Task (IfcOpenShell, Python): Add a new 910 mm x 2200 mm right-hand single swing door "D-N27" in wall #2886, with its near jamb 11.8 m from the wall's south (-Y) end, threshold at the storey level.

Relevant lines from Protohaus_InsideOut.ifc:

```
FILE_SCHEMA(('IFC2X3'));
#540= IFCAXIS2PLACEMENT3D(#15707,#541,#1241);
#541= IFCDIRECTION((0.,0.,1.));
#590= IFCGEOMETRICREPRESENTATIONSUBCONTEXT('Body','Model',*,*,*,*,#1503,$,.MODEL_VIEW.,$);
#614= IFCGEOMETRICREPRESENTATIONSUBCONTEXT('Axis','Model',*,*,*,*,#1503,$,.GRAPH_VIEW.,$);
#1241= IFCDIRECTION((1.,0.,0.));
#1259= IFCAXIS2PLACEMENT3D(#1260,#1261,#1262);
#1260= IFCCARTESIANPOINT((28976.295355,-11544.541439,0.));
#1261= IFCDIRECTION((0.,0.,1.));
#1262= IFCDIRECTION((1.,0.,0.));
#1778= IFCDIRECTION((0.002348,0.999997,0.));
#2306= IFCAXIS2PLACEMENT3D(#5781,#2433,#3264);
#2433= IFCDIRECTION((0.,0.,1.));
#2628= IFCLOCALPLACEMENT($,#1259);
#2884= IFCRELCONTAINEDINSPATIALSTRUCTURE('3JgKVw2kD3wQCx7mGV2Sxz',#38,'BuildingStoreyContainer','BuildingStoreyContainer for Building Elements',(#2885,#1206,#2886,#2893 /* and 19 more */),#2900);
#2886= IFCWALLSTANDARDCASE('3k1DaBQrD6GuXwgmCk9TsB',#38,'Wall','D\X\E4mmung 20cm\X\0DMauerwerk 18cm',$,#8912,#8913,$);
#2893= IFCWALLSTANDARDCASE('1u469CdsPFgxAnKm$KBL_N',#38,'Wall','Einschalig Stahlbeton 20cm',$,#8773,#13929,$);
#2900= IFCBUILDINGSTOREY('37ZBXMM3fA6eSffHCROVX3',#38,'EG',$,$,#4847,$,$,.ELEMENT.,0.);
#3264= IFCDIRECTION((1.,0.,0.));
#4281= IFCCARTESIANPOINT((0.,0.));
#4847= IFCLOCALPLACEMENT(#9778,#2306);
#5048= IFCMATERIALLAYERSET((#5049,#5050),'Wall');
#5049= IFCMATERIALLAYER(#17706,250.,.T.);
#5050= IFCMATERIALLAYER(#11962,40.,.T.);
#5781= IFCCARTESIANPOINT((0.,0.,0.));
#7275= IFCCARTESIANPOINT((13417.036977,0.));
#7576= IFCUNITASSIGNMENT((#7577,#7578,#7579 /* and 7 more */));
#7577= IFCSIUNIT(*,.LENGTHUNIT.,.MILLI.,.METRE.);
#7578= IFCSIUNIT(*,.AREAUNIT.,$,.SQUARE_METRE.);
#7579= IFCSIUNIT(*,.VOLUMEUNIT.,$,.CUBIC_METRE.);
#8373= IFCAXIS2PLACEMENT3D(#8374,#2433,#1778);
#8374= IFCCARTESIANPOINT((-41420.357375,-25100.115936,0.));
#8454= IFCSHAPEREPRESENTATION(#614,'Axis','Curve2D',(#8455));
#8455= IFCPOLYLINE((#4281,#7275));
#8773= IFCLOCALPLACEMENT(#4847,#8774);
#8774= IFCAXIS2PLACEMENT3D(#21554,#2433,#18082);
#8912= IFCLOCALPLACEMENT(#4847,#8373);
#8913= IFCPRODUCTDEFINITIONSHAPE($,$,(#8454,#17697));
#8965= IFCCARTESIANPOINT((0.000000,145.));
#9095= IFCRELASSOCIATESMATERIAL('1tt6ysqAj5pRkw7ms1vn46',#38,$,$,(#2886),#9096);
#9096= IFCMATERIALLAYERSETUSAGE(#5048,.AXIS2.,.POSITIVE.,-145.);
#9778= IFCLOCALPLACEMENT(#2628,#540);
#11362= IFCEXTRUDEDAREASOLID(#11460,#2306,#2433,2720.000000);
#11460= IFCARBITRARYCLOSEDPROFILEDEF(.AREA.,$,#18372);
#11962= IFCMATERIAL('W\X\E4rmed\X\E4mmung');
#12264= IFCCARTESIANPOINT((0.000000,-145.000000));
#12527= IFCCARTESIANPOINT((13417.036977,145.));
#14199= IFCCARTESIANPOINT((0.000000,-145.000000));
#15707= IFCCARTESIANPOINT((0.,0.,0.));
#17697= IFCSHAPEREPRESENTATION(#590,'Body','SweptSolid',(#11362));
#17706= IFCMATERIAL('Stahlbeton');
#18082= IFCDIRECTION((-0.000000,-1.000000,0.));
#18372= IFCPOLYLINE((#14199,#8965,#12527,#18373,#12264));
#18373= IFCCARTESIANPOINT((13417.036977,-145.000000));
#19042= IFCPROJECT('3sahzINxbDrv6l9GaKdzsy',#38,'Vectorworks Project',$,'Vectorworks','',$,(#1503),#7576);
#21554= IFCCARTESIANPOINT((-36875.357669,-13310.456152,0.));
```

```python
import numpy as np
import ifcopenshell
import ifcopenshell.api.feature
import ifcopenshell.api.geometry
import ifcopenshell.api.root
import ifcopenshell.api.spatial
import ifcopenshell.api.type
import ifcopenshell.geom
import ifcopenshell.util.element
import ifcopenshell.util.placement
import ifcopenshell.util.representation
import ifcopenshell.util.shape
import ifcopenshell.util.unit

model = ifcopenshell.open("Protohaus_InsideOut.ifc")
unit_scale = ifcopenshell.util.unit.calculate_unit_scale(model)
settings = ifcopenshell.geom.settings()


def volume(element):
    """Net volume in cubic metres, openings subtracted."""
    shape = ifcopenshell.geom.create_shape(settings, element)
    return ifcopenshell.util.shape.get_volume(shape.geometry)


wall = model.by_guid("3k1DaBQrD6GuXwgmCk9TsB")
storey = ifcopenshell.util.element.get_container(wall, ifc_class="IfcBuildingStorey")
context = ifcopenshell.util.representation.get_context(model, "Model", "Body", "MODEL_VIEW")
before = volume(wall)

width, height, from_end, sill = 0.91, 2.2, 11.8, 0.0  # metres

# The wall runs along its own X axis, and the end named is its -X end.
wall_shape = ifcopenshell.geom.create_shape(settings, wall)
x, y, z = ifcopenshell.util.shape.get_vertices(wall_shape.geometry).T
start = x.min() + from_end
face, thickness = float(y.min()), float(y.max() - y.min())
wall_matrix = ifcopenshell.util.placement.get_local_placement(wall.ObjectPlacement)
level = ifcopenshell.util.placement.get_local_placement(storey.ObjectPlacement)[2, 3]


def in_wall(x, y):
    """Placement at x, y metres in the wall's axes, at sill height."""
    matrix = wall_matrix.copy()
    matrix[:, 3] = wall_matrix @ np.array([x / unit_scale, y / unit_scale, 0.0, 1.0])
    matrix[2, 3] = level + sill / unit_scale
    return matrix


# Opening: a box that overshoots both wall faces by 50 mm.
opening = ifcopenshell.api.root.create_entity(model, ifc_class="IfcOpeningElement")
box = ifcopenshell.api.geometry.add_wall_representation(
    model, context=context, length=width, height=height, thickness=thickness + 0.1
)
ifcopenshell.api.geometry.assign_representation(model, product=opening, representation=box)
ifcopenshell.api.geometry.edit_object_placement(model, product=opening, matrix=in_wall(start, face - 0.05), is_si=False)
ifcopenshell.api.feature.add_feature(model, feature=opening, element=wall)

door = ifcopenshell.api.root.create_entity(model, ifc_class="IfcDoor", name="D-N27")
door.OverallWidth, door.OverallHeight = width / unit_scale, height / unit_scale
body = ifcopenshell.api.geometry.add_door_representation(
    model,
    context=context,
    overall_width=door.OverallWidth,
    overall_height=door.OverallHeight,
    operation_type="SINGLE_SWING_RIGHT",
    lining_properties={"LiningDepth": thickness / unit_scale, "ThresholdDepth": thickness / unit_scale},
)
ifcopenshell.api.geometry.assign_representation(model, product=door, representation=body)
ifcopenshell.api.spatial.assign_container(model, products=[door], relating_structure=storey)
fills = ifcopenshell.api.feature.add_filling(model, opening=opening, element=door)
fills.OwnerHistory = door.OwnerHistory  # required in IFC2X3

# IFC2X3 keeps the operation on the door style.
style = ifcopenshell.api.root.create_entity(model, ifc_class="IfcDoorStyle", name="D-N27")
style.OperationType, style.ConstructionType = "SINGLE_SWING_RIGHT", "NOTDEFINED"
style.ParameterTakesPrecedence = style.Sizeable = False
ifcopenshell.api.type.assign_type(model, related_objects=[door], relating_type=style)

# The lining spans the wall, so the door starts at the wall face.
ifcopenshell.api.geometry.edit_object_placement(model, product=door, matrix=in_wall(start, face), is_si=False)

after = volume(wall)

print(f"wall volume {before:.3f} -> {after:.3f} m3")

model.write("Protohaus_InsideOut_rev.ifc")
```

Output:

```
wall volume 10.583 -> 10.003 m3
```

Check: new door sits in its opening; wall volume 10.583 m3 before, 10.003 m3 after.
